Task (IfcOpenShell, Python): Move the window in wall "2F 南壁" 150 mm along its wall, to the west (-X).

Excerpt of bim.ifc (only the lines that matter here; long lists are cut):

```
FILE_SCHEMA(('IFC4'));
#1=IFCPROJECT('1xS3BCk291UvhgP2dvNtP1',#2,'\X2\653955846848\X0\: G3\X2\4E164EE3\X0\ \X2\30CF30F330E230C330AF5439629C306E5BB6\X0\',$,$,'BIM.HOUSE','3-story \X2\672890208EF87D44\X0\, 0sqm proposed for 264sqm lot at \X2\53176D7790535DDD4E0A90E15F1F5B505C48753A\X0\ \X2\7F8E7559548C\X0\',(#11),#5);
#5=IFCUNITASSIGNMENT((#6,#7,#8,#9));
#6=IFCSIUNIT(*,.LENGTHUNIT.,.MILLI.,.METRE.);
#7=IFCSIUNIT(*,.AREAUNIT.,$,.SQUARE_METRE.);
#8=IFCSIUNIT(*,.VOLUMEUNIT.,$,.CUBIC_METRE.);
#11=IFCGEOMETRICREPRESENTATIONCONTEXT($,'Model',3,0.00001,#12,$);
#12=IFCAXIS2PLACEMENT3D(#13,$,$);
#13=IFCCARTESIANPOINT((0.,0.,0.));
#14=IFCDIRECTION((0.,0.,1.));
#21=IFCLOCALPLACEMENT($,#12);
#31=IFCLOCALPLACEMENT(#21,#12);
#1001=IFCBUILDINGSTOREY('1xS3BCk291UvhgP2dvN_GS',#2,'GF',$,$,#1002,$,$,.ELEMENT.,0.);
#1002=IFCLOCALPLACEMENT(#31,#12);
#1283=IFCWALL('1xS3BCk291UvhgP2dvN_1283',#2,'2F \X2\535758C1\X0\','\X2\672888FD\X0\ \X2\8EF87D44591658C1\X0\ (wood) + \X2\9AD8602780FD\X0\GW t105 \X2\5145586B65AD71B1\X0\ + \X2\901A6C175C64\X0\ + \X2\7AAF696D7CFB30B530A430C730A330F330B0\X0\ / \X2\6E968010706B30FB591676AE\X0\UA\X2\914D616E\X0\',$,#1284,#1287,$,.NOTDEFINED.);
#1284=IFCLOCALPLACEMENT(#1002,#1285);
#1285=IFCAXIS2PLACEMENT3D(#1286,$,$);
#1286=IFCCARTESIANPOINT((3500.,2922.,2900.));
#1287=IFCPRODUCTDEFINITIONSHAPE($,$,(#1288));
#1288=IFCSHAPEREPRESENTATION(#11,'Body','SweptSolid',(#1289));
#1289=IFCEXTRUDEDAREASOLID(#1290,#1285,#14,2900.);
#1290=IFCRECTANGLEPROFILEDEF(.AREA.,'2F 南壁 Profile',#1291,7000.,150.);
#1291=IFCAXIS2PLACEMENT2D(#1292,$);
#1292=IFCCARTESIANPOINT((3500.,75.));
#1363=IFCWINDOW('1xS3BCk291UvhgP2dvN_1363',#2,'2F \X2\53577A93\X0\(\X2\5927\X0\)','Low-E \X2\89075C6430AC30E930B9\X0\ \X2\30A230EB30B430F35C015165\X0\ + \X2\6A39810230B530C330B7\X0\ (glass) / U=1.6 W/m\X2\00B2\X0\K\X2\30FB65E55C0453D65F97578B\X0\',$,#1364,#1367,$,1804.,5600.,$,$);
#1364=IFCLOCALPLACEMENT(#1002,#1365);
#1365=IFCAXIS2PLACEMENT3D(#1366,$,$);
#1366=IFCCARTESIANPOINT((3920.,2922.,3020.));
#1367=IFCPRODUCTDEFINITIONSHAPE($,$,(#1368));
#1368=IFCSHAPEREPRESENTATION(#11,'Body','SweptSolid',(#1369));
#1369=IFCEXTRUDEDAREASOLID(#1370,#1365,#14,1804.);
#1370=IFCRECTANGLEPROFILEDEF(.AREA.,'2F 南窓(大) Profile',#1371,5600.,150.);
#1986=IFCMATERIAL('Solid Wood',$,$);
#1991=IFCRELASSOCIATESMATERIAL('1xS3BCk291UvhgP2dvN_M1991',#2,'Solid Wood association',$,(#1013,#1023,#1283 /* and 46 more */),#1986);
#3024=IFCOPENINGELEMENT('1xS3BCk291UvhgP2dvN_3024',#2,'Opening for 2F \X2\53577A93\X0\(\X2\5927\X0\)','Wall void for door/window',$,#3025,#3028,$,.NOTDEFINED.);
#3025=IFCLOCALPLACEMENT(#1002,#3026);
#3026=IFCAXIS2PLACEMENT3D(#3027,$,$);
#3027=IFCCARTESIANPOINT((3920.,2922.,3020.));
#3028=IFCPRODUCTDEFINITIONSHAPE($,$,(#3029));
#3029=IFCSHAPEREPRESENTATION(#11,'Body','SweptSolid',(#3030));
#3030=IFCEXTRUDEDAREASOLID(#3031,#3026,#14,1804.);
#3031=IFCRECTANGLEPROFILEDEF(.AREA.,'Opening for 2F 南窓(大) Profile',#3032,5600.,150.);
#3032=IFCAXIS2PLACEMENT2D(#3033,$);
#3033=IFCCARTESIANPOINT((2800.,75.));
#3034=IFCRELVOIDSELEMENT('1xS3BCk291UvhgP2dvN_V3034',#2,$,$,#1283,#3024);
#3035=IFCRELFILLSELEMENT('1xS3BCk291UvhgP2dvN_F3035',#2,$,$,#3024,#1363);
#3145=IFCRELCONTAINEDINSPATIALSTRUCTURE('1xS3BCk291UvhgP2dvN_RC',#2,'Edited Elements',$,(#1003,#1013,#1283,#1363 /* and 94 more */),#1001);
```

```python
import ifcopenshell
import ifcopenshell.api.geometry
import ifcopenshell.util.placement
import ifcopenshell.util.unit

model = ifcopenshell.open("bim.ifc")
unit_scale = ifcopenshell.util.unit.calculate_unit_scale(model)

window = model.by_guid("1xS3BCk291UvhgP2dvN_1363")
opening = window.FillsVoids[0].RelatingOpeningElement
wall = opening.VoidsElements[0].RelatingBuildingElement

wall_matrix = ifcopenshell.util.placement.get_local_placement(wall.ObjectPlacement)
shift = wall_matrix[:3, 0] * -0.15 / unit_scale
before = ifcopenshell.util.placement.get_local_placement(window.ObjectPlacement)[:3, 3].copy()

# The window is not placed relative to its opening, so move both.
for product in (opening, window):
    matrix = ifcopenshell.util.placement.get_local_placement(product.ObjectPlacement)
    matrix[:3, 3] += shift
    ifcopenshell.api.geometry.edit_object_placement(model, product=product, matrix=matrix, is_si=False)

after = ifcopenshell.util.placement.get_local_placement(window.ObjectPlacement)[:3, 3]
print("window moved by", (after - before).round(3) + 0.0)

model.write("bim_rev.ifc")
```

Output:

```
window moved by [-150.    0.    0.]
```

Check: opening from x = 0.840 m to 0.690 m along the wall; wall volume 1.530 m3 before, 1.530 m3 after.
